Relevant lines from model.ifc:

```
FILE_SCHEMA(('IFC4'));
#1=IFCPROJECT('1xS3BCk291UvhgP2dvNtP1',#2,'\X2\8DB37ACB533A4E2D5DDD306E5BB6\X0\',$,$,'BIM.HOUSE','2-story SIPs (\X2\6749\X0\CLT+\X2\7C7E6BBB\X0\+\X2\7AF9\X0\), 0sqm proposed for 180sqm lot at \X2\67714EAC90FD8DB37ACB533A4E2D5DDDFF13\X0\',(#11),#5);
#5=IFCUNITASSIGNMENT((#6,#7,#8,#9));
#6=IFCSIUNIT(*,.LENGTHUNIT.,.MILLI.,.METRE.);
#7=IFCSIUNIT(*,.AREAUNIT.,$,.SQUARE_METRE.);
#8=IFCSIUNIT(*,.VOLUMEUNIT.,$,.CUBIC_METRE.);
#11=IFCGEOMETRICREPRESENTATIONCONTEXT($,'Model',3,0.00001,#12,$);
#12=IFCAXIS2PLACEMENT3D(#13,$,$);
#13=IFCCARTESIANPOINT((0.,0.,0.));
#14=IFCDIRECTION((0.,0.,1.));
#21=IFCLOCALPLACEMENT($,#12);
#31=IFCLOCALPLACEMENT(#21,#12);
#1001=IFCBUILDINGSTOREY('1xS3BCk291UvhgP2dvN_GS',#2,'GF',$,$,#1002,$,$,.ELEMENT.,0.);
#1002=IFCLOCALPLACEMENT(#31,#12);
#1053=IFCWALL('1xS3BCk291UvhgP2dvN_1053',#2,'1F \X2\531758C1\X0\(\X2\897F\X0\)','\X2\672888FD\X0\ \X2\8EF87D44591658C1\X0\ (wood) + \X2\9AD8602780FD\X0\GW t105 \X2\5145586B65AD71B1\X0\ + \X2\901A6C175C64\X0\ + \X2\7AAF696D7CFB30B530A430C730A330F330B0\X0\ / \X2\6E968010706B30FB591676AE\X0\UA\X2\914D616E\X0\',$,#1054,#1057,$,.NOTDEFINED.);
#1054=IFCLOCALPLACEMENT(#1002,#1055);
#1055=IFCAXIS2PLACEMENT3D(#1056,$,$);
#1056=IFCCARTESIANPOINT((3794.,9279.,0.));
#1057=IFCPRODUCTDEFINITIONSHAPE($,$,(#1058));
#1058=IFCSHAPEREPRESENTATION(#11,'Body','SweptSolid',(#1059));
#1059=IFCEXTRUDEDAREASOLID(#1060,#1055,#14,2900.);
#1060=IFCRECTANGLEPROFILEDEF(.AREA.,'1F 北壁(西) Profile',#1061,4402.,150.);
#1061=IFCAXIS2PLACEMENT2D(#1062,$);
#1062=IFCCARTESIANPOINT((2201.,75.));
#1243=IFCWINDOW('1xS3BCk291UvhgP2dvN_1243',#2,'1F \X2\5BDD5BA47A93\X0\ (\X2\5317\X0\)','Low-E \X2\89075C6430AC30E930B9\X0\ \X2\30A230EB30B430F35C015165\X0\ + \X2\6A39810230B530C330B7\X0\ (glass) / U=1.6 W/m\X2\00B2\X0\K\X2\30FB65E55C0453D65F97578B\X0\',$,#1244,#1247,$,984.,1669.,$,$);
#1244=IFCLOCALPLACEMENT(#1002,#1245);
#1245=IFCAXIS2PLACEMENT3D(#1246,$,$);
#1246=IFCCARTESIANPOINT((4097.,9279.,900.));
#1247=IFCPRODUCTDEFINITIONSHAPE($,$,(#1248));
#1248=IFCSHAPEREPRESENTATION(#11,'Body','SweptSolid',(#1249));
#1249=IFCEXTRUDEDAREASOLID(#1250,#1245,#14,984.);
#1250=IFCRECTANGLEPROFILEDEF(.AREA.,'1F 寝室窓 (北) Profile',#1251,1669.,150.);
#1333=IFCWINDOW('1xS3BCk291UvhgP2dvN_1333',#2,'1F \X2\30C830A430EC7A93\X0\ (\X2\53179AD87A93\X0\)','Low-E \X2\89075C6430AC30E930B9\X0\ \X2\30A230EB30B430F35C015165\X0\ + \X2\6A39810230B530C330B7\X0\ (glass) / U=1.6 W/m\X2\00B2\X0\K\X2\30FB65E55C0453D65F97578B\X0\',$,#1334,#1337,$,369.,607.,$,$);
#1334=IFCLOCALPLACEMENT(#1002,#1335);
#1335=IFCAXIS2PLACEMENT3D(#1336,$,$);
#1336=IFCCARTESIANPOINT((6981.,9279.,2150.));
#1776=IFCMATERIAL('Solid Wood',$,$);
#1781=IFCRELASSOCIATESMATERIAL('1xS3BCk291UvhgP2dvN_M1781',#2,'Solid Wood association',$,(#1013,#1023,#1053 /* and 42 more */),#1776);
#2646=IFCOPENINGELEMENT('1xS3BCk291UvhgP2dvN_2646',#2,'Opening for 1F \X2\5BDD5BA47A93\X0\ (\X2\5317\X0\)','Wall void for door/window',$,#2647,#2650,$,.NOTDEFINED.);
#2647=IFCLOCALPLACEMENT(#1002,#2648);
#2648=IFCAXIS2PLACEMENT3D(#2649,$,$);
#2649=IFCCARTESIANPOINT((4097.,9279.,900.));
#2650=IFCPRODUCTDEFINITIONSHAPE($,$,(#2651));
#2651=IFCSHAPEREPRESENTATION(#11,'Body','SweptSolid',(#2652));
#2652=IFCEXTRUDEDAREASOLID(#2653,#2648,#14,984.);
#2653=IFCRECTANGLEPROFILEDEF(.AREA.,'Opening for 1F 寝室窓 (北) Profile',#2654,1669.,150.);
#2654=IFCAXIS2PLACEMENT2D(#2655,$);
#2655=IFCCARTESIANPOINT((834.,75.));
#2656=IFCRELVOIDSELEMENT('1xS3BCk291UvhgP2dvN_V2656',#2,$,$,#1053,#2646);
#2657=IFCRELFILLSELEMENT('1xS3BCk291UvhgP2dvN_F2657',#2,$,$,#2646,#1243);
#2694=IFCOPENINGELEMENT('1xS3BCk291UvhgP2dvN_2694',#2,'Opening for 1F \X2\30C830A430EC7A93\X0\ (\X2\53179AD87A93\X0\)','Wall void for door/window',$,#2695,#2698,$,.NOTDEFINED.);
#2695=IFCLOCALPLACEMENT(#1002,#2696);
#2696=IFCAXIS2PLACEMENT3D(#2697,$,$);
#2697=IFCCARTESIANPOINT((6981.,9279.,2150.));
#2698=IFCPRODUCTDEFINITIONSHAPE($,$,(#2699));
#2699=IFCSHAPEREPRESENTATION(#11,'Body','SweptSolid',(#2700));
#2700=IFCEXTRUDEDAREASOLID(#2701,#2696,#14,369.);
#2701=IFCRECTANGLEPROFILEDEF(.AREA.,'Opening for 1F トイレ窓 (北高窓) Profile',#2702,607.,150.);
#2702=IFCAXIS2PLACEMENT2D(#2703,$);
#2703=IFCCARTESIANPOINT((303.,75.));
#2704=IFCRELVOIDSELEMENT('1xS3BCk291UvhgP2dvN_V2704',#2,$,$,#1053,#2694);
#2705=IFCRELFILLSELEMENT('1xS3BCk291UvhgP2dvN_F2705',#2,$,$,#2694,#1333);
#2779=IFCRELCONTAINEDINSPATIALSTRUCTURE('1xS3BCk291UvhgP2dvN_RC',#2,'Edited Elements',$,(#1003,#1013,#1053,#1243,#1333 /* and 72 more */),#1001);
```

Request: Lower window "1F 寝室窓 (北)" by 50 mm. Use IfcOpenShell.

```python
import numpy as np
import ifcopenshell
import ifcopenshell.api.geometry
import ifcopenshell.util.placement
import ifcopenshell.util.unit

model = ifcopenshell.open("model.ifc")
unit_scale = ifcopenshell.util.unit.calculate_unit_scale(model)

window = model.by_guid("1xS3BCk291UvhgP2dvN_1243")
opening = window.FillsVoids[0].RelatingOpeningElement
dz = -0.05 / unit_scale

shift = np.array([0.0, 0.0, dz])
# The window is not placed relative to its opening, so move both.
for product in (opening, window):
    matrix = ifcopenshell.util.placement.get_local_placement(product.ObjectPlacement)
    matrix[:3, 3] += shift
    ifcopenshell.api.geometry.edit_object_placement(model, product=product, matrix=matrix, is_si=False)

print(f"moved by {dz * unit_scale:+.3f} m")

model.write("model_rev.ifc")
```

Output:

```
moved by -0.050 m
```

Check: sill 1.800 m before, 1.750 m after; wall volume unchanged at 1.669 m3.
